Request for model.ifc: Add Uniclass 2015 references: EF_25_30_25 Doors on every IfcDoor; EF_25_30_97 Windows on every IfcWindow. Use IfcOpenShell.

First a look at what the model holds.

```python
import ifcopenshell

model = ifcopenshell.open("model.ifc")
print(model.schema)
print("classifications:", [c.Name for c in model.by_type("IfcClassification")])
for ifc_class in ("IfcDoor", "IfcRoof", "IfcStair", "IfcWall", "IfcWindow"):
    print(ifc_class, len(model.by_type(ifc_class)))
```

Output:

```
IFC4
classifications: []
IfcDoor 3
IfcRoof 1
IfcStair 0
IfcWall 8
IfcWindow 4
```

```python
import ifcopenshell
import ifcopenshell.api.classification

model = ifcopenshell.open("model.ifc")

system = ifcopenshell.api.classification.add_classification(model, classification="Uniclass 2015")

codes = {
    "IfcDoor": ("EF_25_30_25", "Doors"),
    "IfcWindow": ("EF_25_30_97", "Windows"),
}
for ifc_class, (code, name) in codes.items():
    products = model.by_type(ifc_class)
    ifcopenshell.api.classification.add_reference(
        model, products=products, classification=system, identification=code, name=name
    )
    print(code, len(products))

model.write("model_updated.ifc")
```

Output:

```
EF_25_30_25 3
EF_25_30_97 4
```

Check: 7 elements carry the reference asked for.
